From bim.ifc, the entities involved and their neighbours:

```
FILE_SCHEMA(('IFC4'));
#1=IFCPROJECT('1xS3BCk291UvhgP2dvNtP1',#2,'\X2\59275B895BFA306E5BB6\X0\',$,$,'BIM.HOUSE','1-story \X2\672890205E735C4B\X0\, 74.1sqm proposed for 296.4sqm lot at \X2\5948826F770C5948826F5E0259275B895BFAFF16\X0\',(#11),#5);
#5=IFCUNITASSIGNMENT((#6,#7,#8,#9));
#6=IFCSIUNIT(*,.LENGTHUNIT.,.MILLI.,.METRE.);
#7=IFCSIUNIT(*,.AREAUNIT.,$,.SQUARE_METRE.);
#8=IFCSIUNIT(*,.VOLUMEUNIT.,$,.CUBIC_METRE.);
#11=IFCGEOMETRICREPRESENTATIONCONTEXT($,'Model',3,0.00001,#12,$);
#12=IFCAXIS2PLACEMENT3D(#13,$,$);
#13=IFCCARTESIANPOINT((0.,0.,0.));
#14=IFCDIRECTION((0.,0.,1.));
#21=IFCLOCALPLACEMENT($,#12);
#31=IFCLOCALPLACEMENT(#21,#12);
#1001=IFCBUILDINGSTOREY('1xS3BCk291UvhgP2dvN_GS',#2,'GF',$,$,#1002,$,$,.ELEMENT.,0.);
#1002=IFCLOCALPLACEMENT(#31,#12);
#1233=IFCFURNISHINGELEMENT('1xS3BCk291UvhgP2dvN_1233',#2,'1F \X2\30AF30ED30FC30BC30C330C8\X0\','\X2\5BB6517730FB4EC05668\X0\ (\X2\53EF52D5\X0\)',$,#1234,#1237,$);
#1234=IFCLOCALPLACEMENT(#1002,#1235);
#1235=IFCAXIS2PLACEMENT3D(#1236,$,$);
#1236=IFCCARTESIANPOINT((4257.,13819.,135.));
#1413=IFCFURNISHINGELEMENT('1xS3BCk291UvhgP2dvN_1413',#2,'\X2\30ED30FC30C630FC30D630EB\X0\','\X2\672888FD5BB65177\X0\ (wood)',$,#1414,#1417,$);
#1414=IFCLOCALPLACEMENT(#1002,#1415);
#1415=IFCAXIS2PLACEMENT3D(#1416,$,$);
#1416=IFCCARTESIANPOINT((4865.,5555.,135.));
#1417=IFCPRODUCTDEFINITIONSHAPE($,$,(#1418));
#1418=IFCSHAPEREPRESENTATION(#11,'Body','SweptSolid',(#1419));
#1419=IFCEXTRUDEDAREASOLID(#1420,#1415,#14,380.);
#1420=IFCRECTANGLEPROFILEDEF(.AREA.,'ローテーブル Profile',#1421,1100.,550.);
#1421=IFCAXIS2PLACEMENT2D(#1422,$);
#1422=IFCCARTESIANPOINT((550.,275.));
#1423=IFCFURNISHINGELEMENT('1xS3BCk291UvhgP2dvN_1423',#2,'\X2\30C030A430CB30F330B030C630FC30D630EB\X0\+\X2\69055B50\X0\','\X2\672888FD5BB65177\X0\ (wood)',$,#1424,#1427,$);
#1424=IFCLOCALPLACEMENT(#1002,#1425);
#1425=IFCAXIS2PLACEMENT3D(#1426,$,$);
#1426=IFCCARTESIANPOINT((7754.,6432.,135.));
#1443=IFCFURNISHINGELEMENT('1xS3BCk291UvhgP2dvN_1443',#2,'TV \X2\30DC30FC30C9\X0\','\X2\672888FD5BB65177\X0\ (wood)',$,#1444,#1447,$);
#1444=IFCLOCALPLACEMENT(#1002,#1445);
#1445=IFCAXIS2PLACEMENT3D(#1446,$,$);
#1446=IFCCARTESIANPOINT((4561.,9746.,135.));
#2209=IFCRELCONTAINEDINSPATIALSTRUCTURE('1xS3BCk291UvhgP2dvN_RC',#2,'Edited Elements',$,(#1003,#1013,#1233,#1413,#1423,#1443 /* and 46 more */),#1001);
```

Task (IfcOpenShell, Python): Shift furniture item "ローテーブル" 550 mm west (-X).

```python
import ifcopenshell
import ifcopenshell.api.geometry
import ifcopenshell.util.placement

model = ifcopenshell.open("bim.ifc")

item = model.by_guid("1xS3BCk291UvhgP2dvN_1413")
matrix = ifcopenshell.util.placement.get_local_placement(item.ObjectPlacement)
matrix[0, 3] -= 550.0
ifcopenshell.api.geometry.edit_object_placement(model, product=item, matrix=matrix, is_si=False)

print(ifcopenshell.util.placement.get_local_placement(item.ObjectPlacement).round(3) + 0.0)

model.write("bim-out.ifc")
```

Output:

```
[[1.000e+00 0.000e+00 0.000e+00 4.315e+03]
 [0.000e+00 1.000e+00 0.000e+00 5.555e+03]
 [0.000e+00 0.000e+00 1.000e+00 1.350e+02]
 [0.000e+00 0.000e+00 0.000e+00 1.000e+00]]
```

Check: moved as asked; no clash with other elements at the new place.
